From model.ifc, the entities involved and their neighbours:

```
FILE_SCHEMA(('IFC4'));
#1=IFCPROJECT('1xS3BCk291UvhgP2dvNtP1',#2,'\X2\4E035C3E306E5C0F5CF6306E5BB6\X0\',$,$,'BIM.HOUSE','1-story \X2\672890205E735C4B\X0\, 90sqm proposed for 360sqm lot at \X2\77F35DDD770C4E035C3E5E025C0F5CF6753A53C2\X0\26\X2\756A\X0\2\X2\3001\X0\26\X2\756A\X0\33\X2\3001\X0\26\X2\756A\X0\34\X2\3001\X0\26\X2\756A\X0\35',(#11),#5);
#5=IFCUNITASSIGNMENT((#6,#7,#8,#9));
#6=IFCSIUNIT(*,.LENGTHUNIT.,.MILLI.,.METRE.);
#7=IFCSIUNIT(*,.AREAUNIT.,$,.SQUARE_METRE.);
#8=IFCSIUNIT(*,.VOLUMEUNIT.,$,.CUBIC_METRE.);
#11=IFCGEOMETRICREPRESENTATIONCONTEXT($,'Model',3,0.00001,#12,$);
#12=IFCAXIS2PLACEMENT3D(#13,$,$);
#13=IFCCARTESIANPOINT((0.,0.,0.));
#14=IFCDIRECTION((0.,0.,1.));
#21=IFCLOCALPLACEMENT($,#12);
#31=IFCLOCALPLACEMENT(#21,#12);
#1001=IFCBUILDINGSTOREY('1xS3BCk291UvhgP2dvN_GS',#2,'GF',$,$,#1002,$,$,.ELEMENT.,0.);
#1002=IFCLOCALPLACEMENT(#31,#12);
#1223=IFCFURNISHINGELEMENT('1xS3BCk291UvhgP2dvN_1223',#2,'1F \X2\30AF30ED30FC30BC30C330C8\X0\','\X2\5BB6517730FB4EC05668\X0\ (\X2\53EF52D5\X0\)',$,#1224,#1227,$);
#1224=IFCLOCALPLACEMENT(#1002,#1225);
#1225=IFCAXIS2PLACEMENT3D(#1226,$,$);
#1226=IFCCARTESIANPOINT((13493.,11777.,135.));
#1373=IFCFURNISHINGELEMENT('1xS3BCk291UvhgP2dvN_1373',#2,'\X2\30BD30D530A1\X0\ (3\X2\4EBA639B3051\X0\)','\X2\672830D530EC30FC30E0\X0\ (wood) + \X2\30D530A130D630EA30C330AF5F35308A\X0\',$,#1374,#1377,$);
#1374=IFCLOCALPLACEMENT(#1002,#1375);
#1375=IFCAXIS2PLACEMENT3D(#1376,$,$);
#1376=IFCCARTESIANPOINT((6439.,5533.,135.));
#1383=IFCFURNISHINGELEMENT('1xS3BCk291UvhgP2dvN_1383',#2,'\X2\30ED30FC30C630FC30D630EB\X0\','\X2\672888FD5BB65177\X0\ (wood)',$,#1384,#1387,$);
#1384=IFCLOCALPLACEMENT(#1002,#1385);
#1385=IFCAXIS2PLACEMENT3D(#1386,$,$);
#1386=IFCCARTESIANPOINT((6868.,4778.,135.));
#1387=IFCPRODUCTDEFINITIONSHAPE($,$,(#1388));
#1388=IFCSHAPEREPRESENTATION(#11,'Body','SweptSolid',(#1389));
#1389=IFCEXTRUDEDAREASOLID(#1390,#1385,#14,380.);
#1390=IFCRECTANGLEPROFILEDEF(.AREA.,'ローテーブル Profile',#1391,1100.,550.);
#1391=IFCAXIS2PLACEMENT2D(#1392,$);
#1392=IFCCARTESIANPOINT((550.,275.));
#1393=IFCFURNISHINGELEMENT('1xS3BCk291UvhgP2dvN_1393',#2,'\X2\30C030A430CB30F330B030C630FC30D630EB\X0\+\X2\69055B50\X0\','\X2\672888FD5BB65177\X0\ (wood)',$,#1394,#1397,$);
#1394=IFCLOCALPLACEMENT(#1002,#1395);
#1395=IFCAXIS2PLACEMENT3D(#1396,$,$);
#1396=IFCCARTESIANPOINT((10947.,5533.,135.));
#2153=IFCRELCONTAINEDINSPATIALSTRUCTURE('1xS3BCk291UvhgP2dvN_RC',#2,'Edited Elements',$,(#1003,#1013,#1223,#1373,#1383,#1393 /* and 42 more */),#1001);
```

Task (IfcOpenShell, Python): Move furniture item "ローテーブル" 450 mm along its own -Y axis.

```python
import ifcopenshell
import ifcopenshell.api.geometry
import ifcopenshell.util.placement
import ifcopenshell.util.unit

model = ifcopenshell.open("model.ifc")
unit_scale = ifcopenshell.util.unit.calculate_unit_scale(model)

item = model.by_guid("1xS3BCk291UvhgP2dvN_1383")
matrix = ifcopenshell.util.placement.get_local_placement(item.ObjectPlacement)
matrix[:3, 3] -= matrix[:3, 1] * 0.45 / unit_scale
ifcopenshell.api.geometry.edit_object_placement(model, product=item, matrix=matrix, is_si=False)

print(ifcopenshell.util.placement.get_local_placement(item.ObjectPlacement).round(3) + 0.0)

model.write("model_rev.ifc")
```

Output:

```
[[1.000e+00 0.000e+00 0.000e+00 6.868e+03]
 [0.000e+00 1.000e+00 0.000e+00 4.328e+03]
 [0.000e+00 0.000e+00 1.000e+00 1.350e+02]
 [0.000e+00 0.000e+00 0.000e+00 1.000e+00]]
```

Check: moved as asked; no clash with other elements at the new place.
